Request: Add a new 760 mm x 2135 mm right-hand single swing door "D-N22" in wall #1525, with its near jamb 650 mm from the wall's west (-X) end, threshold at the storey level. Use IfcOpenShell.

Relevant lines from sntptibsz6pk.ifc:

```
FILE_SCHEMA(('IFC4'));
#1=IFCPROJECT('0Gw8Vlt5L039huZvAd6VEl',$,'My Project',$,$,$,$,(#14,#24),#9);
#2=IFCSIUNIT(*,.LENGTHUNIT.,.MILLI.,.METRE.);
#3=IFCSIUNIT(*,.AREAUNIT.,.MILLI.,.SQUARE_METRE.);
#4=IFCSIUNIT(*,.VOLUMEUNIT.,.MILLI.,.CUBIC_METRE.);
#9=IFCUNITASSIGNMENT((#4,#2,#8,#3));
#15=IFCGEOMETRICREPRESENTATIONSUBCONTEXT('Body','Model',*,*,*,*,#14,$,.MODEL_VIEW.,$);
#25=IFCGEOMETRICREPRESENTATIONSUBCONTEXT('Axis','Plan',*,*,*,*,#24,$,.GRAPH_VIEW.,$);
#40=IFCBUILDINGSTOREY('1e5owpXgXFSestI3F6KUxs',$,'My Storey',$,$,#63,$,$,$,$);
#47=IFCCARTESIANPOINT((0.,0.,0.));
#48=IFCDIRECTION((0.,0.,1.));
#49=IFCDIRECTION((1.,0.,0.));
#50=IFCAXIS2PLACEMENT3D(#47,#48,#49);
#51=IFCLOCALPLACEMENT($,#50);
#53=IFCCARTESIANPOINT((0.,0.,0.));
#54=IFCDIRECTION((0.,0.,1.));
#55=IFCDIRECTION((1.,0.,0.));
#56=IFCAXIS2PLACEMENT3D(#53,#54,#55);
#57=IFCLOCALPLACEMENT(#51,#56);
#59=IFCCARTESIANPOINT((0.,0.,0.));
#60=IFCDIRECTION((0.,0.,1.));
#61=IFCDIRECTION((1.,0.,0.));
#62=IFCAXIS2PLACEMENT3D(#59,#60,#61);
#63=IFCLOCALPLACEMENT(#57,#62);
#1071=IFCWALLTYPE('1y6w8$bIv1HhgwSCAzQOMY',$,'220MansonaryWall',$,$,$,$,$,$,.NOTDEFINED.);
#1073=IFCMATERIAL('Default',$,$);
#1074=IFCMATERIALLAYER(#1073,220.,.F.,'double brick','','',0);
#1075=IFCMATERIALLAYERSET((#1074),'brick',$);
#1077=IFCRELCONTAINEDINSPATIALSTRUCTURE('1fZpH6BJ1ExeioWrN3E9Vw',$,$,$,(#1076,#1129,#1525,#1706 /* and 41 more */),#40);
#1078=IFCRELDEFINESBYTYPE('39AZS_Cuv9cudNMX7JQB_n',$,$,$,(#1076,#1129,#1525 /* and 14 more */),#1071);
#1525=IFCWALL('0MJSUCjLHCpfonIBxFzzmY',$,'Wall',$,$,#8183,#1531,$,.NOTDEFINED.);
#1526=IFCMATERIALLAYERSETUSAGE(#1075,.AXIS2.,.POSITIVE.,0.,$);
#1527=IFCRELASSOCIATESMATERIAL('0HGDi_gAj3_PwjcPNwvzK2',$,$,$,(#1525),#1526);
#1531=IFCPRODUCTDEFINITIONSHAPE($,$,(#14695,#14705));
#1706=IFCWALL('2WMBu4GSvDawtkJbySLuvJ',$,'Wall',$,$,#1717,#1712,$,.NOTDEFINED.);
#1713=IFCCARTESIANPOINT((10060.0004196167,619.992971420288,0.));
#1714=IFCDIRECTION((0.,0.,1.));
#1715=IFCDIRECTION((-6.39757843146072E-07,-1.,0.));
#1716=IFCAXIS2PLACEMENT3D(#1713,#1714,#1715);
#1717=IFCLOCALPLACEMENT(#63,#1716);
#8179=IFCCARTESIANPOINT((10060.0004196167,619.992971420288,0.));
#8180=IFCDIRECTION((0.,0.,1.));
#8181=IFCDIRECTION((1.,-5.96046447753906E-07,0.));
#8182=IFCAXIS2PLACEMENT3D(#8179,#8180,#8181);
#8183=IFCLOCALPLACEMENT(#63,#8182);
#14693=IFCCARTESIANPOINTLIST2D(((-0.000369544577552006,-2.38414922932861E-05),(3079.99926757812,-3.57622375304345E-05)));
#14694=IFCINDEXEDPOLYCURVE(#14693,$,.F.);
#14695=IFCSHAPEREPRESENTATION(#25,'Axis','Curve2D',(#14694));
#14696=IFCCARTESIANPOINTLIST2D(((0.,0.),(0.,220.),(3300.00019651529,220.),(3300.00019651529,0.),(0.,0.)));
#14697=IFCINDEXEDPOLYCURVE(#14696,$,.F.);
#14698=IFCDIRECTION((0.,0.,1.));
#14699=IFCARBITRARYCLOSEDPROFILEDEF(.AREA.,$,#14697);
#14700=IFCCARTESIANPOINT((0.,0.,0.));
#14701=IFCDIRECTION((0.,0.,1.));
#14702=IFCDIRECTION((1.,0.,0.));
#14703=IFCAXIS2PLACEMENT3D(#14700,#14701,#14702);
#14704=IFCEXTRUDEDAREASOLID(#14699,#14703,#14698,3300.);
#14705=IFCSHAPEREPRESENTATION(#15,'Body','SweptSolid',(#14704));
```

```python
import numpy as np
import ifcopenshell
import ifcopenshell.api.feature
import ifcopenshell.api.geometry
import ifcopenshell.api.root
import ifcopenshell.api.spatial
import ifcopenshell.geom
import ifcopenshell.util.element
import ifcopenshell.util.placement
import ifcopenshell.util.representation
import ifcopenshell.util.shape
import ifcopenshell.util.unit

model = ifcopenshell.open("sntptibsz6pk.ifc")
unit_scale = ifcopenshell.util.unit.calculate_unit_scale(model)
settings = ifcopenshell.geom.settings()


def volume(element):
    """Net volume in cubic metres, openings subtracted."""
    shape = ifcopenshell.geom.create_shape(settings, element)
    return ifcopenshell.util.shape.get_volume(shape.geometry)


wall = model.by_guid("0MJSUCjLHCpfonIBxFzzmY")
storey = ifcopenshell.util.element.get_container(wall, ifc_class="IfcBuildingStorey")
context = ifcopenshell.util.representation.get_context(model, "Model", "Body", "MODEL_VIEW")
before = volume(wall)

width, height, from_end, sill = 0.76, 2.135, 0.65, 0.0  # metres

# The wall runs along its own X axis, and the end named is its -X end.
wall_shape = ifcopenshell.geom.create_shape(settings, wall)
x, y, z = ifcopenshell.util.shape.get_vertices(wall_shape.geometry).T
start = x.min() + from_end
face, thickness = float(y.min()), float(y.max() - y.min())
wall_matrix = ifcopenshell.util.placement.get_local_placement(wall.ObjectPlacement)
level = ifcopenshell.util.placement.get_local_placement(storey.ObjectPlacement)[2, 3]


def in_wall(x, y):
    """Placement at x, y metres in the wall's axes, at sill height."""
    matrix = wall_matrix.copy()
    matrix[:, 3] = wall_matrix @ np.array([x / unit_scale, y / unit_scale, 0.0, 1.0])
    matrix[2, 3] = level + sill / unit_scale
    return matrix


# Opening: a box that overshoots both wall faces by 50 mm.
opening = ifcopenshell.api.root.create_entity(model, ifc_class="IfcOpeningElement", predefined_type="OPENING")
box = ifcopenshell.api.geometry.add_wall_representation(
    model, context=context, length=width, height=height, thickness=thickness + 0.1
)
ifcopenshell.api.geometry.assign_representation(model, product=opening, representation=box)
ifcopenshell.api.geometry.edit_object_placement(model, product=opening, matrix=in_wall(start, face - 0.05), is_si=False)
ifcopenshell.api.feature.add_feature(model, feature=opening, element=wall)

door = ifcopenshell.api.root.create_entity(model, ifc_class="IfcDoor", name="D-N22", predefined_type="DOOR")
door.OverallWidth, door.OverallHeight = width / unit_scale, height / unit_scale
door.OperationType = "SINGLE_SWING_RIGHT"
body = ifcopenshell.api.geometry.add_door_representation(
    model,
    context=context,
    overall_width=door.OverallWidth,
    overall_height=door.OverallHeight,
    operation_type="SINGLE_SWING_RIGHT",
    lining_properties={"LiningDepth": thickness / unit_scale, "ThresholdDepth": thickness / unit_scale},
)
ifcopenshell.api.geometry.assign_representation(model, product=door, representation=body)
ifcopenshell.api.spatial.assign_container(model, products=[door], relating_structure=storey)
ifcopenshell.api.feature.add_filling(model, opening=opening, element=door)

# The lining spans the wall, so the door starts at the wall face.
ifcopenshell.api.geometry.edit_object_placement(model, product=door, matrix=in_wall(start, face), is_si=False)

after = volume(wall)

print(f"wall volume {before:.3f} -> {after:.3f} m3")

model.write("sntptibsz6pk_updated.ifc")
```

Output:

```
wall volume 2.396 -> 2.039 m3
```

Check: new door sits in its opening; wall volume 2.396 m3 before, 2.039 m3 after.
